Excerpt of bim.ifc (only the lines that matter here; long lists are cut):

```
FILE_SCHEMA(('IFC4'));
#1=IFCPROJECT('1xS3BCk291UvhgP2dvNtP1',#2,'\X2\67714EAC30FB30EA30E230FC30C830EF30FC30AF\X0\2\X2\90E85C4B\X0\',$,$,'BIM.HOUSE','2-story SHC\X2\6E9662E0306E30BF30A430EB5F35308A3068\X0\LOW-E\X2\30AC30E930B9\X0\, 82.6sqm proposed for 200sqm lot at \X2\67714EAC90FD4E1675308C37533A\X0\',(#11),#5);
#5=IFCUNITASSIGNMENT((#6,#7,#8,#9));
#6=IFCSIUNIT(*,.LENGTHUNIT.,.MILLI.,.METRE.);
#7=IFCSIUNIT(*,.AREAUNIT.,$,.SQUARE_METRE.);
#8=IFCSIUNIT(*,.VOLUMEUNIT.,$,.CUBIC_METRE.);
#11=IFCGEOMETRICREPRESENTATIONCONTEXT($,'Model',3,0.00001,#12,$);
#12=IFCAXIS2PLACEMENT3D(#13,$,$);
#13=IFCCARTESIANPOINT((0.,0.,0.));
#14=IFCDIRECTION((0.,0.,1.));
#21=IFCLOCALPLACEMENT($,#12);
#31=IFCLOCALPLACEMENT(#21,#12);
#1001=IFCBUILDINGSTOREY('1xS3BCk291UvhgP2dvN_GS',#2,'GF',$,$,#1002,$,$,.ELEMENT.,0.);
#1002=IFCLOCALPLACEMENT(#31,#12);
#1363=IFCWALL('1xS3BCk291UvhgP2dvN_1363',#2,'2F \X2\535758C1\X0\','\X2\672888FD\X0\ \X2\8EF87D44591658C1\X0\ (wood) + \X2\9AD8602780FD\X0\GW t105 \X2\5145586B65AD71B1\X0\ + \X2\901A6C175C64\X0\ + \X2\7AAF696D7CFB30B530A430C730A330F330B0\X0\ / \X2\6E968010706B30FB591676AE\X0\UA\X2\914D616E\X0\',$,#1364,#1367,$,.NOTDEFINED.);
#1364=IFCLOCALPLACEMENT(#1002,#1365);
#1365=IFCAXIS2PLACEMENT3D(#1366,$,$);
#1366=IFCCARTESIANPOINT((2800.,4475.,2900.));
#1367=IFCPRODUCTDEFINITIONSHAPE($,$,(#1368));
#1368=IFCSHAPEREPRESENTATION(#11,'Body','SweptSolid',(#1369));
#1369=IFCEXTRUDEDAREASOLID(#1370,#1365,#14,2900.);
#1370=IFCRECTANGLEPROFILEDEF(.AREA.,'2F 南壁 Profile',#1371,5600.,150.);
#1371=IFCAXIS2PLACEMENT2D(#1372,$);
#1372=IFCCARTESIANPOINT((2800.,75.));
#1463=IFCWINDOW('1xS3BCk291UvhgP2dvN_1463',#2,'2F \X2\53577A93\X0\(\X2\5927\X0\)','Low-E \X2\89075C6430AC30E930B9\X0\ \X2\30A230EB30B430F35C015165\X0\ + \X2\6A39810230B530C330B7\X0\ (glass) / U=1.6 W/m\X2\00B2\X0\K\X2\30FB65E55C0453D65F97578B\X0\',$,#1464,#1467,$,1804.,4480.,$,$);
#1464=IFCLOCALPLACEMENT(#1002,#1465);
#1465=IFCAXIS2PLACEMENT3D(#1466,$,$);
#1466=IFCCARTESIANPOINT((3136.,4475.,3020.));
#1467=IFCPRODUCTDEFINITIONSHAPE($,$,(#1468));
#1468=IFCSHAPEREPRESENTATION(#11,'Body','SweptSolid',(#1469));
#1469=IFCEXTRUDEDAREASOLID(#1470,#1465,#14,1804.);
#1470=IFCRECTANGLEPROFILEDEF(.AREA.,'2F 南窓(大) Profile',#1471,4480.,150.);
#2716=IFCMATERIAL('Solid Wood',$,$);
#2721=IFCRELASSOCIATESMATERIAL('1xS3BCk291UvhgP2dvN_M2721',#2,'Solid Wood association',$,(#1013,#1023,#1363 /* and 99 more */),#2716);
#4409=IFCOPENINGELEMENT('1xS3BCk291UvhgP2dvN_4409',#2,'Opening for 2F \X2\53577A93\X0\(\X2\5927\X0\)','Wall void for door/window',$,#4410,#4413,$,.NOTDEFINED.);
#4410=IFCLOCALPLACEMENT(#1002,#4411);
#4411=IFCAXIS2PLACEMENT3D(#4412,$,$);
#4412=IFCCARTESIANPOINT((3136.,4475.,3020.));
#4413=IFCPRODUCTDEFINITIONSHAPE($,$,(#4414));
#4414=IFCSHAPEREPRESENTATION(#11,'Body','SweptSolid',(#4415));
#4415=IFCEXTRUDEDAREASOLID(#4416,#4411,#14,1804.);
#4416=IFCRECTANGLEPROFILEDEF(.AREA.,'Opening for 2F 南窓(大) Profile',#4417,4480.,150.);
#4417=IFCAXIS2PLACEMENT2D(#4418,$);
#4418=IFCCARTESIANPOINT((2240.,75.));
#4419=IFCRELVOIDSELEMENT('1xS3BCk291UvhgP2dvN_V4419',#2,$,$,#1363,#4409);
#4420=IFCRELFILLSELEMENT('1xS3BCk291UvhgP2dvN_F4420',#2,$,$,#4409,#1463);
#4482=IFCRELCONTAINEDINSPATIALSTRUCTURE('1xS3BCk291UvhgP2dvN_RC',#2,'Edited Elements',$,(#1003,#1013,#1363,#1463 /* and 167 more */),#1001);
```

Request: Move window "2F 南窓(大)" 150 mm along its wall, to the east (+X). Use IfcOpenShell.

```python
import ifcopenshell
import ifcopenshell.api.geometry
import ifcopenshell.util.placement
import ifcopenshell.util.unit

model = ifcopenshell.open("bim.ifc")
unit_scale = ifcopenshell.util.unit.calculate_unit_scale(model)

window = model.by_guid("1xS3BCk291UvhgP2dvN_1463")
opening = window.FillsVoids[0].RelatingOpeningElement
wall = opening.VoidsElements[0].RelatingBuildingElement

wall_matrix = ifcopenshell.util.placement.get_local_placement(wall.ObjectPlacement)
shift = wall_matrix[:3, 0] * 0.15 / unit_scale
before = ifcopenshell.util.placement.get_local_placement(window.ObjectPlacement)[:3, 3].copy()

# The window is not placed relative to its opening, so move both.
for product in (opening, window):
    matrix = ifcopenshell.util.placement.get_local_placement(product.ObjectPlacement)
    matrix[:3, 3] += shift
    ifcopenshell.api.geometry.edit_object_placement(model, product=product, matrix=matrix, is_si=False)

after = ifcopenshell.util.placement.get_local_placement(window.ObjectPlacement)[:3, 3]
print("window moved by", (after - before).round(3) + 0.0)

model.write("bim-out.ifc")
```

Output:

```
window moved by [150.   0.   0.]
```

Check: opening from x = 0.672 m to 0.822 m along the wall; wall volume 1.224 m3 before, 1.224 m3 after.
